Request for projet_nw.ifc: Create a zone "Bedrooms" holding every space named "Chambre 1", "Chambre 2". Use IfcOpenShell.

First a look at what the model holds.

```python
import ifcopenshell

model = ifcopenshell.open("projet_nw.ifc")
print(model.schema)
seen = {}
for space in model.by_type("IfcSpace"):
    seen[space.LongName] = seen.get(space.LongName, 0) + 1
for name, count in sorted(seen.items(), key=str):
    print(count, "x", name)
print("zones:", [z.Name for z in model.by_type("IfcZone")][:20])
```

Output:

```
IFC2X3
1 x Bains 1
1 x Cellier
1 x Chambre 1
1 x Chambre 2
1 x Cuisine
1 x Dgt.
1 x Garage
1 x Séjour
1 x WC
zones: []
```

```python
import ifcopenshell
import ifcopenshell.api.group
import ifcopenshell.api.root

model = ifcopenshell.open("projet_nw.ifc")

names = {"Chambre 1", "Chambre 2"}
spaces = [s for s in model.by_type("IfcSpace") if s.LongName in names]

zone = ifcopenshell.api.root.create_entity(model, ifc_class="IfcZone", name="Bedrooms")
ifcopenshell.api.group.assign_group(model, products=spaces, group=zone)
print(len(spaces), "spaces in", zone.Name)

model.write("projet_nw_rev.ifc")
```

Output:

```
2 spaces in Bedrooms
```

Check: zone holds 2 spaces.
